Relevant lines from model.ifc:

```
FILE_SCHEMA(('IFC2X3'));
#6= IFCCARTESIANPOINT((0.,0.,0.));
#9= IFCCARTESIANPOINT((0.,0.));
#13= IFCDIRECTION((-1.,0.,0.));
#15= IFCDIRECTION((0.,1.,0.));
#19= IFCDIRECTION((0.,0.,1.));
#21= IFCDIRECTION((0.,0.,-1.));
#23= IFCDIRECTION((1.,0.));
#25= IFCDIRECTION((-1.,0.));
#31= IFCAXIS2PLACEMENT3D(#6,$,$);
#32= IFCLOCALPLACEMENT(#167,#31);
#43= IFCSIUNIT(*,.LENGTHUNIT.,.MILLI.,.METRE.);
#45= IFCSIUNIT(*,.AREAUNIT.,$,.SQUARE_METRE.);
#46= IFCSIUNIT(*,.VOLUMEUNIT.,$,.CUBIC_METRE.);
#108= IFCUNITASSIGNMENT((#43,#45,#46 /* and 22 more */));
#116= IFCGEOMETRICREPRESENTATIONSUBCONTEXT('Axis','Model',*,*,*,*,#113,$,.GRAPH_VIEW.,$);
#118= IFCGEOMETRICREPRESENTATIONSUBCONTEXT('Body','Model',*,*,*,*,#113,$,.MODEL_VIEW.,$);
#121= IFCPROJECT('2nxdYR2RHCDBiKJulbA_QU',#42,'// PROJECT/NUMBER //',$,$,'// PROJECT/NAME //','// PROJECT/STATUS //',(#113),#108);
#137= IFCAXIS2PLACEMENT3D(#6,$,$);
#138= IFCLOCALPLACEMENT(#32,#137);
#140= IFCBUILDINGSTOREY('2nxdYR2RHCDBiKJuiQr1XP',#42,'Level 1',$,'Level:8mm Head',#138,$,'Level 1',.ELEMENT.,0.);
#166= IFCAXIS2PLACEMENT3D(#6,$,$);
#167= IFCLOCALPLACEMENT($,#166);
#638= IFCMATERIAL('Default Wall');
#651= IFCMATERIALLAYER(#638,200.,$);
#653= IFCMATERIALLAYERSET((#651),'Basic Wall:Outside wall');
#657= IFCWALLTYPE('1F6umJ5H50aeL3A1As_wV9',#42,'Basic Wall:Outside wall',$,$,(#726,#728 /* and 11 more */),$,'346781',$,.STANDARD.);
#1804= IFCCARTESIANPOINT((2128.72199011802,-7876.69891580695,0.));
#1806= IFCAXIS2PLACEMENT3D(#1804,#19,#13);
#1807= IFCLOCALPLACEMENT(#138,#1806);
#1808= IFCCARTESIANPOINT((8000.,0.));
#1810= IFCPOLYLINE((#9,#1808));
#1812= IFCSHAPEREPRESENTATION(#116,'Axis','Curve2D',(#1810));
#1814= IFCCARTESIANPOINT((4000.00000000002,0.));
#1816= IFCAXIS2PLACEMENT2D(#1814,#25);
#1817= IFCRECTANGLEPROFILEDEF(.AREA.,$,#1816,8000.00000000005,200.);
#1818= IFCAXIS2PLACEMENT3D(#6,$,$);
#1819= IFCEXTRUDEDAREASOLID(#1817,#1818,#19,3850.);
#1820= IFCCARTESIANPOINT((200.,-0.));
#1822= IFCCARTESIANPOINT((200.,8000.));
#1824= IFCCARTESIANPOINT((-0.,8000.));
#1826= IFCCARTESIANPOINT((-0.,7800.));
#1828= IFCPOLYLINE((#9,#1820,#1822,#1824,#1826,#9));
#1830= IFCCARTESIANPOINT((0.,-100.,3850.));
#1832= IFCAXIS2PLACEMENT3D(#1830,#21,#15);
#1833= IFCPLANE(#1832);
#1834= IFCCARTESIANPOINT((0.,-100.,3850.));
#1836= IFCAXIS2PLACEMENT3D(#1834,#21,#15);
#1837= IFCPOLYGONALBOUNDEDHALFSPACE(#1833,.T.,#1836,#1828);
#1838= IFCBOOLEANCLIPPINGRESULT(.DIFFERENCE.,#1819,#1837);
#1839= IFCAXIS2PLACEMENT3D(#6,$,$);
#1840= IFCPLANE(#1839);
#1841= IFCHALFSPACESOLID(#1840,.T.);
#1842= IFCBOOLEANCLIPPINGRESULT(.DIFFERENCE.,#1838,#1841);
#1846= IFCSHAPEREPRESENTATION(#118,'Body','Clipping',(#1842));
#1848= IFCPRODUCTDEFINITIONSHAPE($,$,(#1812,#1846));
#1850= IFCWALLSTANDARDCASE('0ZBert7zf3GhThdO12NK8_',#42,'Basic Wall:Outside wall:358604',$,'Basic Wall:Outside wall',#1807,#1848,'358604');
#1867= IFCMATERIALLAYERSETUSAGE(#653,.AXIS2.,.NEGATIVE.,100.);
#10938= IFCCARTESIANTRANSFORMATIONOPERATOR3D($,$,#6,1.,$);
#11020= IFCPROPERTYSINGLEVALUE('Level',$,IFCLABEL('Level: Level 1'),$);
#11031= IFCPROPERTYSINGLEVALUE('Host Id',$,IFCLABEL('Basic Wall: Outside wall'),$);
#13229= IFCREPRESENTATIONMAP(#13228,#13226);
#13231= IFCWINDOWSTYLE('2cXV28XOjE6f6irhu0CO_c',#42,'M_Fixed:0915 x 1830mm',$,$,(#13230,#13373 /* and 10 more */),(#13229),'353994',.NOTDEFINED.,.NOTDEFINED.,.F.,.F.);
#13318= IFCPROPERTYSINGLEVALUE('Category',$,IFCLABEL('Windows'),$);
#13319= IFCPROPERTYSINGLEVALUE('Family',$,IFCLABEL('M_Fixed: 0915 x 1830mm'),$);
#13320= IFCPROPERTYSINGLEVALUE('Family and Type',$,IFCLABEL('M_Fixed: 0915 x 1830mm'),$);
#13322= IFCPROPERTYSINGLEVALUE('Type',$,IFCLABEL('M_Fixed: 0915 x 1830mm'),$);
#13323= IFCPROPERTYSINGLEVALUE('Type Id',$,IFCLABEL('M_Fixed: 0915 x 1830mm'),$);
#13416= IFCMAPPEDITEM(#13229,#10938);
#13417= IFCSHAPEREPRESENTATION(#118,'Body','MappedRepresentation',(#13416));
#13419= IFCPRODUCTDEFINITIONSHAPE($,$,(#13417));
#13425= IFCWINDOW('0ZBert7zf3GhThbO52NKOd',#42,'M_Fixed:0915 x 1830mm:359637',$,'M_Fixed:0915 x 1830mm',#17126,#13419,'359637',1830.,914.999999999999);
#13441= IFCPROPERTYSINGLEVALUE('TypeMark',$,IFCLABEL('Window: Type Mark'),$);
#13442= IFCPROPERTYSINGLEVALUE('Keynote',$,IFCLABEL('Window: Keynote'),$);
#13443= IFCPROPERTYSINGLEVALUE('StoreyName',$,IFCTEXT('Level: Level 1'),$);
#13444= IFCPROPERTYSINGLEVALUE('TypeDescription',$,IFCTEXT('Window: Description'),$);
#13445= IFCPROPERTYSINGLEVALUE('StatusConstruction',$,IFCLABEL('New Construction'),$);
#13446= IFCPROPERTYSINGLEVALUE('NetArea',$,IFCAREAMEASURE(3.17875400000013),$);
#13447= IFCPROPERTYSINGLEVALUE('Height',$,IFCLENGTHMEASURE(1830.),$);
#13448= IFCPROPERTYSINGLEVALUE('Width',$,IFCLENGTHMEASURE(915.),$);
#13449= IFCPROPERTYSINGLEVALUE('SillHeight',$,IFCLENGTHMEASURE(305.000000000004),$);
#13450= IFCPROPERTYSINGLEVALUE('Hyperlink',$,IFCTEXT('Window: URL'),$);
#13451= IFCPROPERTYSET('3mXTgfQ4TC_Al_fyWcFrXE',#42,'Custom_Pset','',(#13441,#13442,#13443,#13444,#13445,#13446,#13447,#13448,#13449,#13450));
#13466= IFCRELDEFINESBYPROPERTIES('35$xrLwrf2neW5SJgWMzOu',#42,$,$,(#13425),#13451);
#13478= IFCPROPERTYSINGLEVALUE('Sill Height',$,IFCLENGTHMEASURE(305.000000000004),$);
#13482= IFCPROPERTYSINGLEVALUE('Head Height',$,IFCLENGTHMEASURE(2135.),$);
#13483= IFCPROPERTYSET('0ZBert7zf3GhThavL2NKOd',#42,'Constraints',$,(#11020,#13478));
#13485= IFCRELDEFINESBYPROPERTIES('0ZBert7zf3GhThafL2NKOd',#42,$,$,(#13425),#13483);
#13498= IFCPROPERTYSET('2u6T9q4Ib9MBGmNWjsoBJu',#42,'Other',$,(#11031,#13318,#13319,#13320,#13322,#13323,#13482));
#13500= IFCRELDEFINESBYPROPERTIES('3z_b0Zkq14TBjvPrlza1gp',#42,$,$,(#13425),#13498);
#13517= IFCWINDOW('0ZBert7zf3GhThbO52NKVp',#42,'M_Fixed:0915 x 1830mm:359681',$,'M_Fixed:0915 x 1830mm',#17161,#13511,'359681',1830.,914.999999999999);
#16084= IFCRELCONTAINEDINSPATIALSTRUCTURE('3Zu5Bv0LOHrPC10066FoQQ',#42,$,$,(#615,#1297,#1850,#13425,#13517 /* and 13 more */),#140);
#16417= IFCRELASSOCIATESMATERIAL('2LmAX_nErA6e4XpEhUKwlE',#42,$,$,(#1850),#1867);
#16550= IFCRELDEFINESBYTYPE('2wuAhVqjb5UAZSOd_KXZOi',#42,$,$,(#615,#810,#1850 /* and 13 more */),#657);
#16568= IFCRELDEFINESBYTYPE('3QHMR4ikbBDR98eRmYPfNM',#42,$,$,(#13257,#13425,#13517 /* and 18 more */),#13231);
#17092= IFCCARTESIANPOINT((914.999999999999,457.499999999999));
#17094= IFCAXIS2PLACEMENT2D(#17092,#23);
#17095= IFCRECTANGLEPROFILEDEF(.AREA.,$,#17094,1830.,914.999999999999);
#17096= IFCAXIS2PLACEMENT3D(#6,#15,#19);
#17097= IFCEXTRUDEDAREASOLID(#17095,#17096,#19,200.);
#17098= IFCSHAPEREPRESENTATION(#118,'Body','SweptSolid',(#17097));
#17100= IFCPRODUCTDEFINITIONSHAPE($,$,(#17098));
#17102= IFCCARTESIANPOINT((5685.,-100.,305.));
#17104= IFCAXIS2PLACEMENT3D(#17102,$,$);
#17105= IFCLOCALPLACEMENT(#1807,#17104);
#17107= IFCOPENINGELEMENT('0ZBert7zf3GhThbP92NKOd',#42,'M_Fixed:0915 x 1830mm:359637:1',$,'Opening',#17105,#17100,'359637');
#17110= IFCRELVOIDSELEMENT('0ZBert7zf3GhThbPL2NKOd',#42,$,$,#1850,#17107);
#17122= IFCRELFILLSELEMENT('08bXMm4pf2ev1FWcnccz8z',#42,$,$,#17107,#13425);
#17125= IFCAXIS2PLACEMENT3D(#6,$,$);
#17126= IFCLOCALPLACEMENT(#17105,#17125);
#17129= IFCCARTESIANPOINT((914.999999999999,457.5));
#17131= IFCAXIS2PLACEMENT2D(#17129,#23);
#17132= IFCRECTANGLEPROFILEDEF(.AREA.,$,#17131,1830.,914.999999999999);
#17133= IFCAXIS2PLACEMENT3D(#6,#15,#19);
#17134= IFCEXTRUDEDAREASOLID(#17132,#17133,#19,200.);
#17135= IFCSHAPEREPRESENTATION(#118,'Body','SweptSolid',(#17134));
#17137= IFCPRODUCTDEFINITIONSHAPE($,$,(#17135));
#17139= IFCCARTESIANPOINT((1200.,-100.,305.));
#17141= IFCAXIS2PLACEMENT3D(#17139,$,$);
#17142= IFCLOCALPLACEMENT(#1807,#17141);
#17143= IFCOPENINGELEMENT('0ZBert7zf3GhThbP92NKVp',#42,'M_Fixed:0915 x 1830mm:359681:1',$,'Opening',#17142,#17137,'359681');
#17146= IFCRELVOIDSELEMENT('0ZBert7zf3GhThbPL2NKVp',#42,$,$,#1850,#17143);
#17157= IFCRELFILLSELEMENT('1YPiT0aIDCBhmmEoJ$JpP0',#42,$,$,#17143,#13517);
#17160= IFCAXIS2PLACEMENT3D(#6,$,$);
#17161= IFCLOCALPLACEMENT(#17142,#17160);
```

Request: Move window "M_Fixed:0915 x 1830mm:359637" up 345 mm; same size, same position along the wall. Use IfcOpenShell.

```python
import numpy as np
import ifcopenshell
import ifcopenshell.api.geometry
import ifcopenshell.api.pset
import ifcopenshell.util.element
import ifcopenshell.util.placement
import ifcopenshell.util.unit

model = ifcopenshell.open("model.ifc")
unit_scale = ifcopenshell.util.unit.calculate_unit_scale(model)

window = model.by_guid("0ZBert7zf3GhThbO52NKOd")
opening = window.FillsVoids[0].RelatingOpeningElement
dz = 345.0

shift = np.array([0.0, 0.0, dz])
# The window is placed relative to its opening, so it follows when the opening moves.
matrix = ifcopenshell.util.placement.get_local_placement(opening.ObjectPlacement)
matrix[:3, 3] += shift
ifcopenshell.api.geometry.edit_object_placement(
    model, product=opening, matrix=matrix, is_si=False, should_transform_children=True
)

# Keep the stored heights in step.
pset = model.by_id(ifcopenshell.util.element.get_pset(window, "Custom_Pset", should_inherit=False)["id"])
ifcopenshell.api.pset.edit_pset(model, pset=pset, properties={
    "SillHeight": model.create_entity("IfcLengthMeasure", ifcopenshell.util.element.get_pset(window, "Constraints", "Sill Height") + dz),
})
pset = model.by_id(ifcopenshell.util.element.get_pset(window, "Constraints", should_inherit=False)["id"])
ifcopenshell.api.pset.edit_pset(model, pset=pset, properties={
    "Sill Height": model.create_entity("IfcLengthMeasure", ifcopenshell.util.element.get_pset(window, "Constraints", "Sill Height") + dz),
})
pset = model.by_id(ifcopenshell.util.element.get_pset(window, "Other", should_inherit=False)["id"])
ifcopenshell.api.pset.edit_pset(model, pset=pset, properties={
    "Head Height": model.create_entity("IfcLengthMeasure", ifcopenshell.util.element.get_pset(window, "Other", "Head Height") + dz),
})

print(f"moved by {dz * unit_scale:+.3f} m")

model.write("model_updated.ifc")
```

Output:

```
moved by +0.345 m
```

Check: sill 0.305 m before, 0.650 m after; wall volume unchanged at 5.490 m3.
